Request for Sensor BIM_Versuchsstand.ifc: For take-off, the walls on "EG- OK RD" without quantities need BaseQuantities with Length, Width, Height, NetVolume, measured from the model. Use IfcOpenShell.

First a look at what the model holds.

```python
import ifcopenshell
import ifcopenshell.util.element
import ifcopenshell.util.unit

model = ifcopenshell.open("Sensor BIM_Versuchsstand.ifc")
print(model.schema)
for unit_type in ("LENGTHUNIT", "AREAUNIT", "VOLUMEUNIT"):
    print(unit_type, ifcopenshell.util.unit.calculate_unit_scale(model, unit_type))
storey = next(s for s in model.by_type("IfcBuildingStorey") if s.Name == "EG- OK RD")
walls = [e for e in ifcopenshell.util.element.get_decomposition(storey) if e.is_a("IfcWall")]
for e in sorted(walls, key=lambda e: e.id()):
    print(e.id(), e.is_a(), e.Name, list(ifcopenshell.util.element.get_psets(e, qtos_only=True)), sep=" | ")
```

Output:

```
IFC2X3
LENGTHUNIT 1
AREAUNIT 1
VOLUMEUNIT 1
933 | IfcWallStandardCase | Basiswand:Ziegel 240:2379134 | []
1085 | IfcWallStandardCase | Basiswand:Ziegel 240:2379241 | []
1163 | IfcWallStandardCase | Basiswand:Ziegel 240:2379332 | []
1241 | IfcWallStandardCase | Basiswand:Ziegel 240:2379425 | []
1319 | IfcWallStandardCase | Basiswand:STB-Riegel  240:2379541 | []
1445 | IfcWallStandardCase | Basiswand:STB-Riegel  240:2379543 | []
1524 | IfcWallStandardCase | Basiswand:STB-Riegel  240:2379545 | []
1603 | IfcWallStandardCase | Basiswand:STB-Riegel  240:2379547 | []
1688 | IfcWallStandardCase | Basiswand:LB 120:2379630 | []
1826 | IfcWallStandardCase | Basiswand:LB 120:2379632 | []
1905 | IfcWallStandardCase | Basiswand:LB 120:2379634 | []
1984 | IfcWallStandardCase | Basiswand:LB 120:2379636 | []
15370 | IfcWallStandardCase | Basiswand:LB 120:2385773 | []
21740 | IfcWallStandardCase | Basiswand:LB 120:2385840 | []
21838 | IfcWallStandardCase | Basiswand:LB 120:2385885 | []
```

```python
import ifcopenshell
import ifcopenshell.api.pset
import ifcopenshell.geom
import ifcopenshell.util.element
import ifcopenshell.util.shape
import ifcopenshell.util.unit

model = ifcopenshell.open("Sensor BIM_Versuchsstand.ifc")
unit_scale = ifcopenshell.util.unit.calculate_unit_scale(model)
volume_scale = ifcopenshell.util.unit.calculate_unit_scale(model, "VOLUMEUNIT")
settings = ifcopenshell.geom.settings()

storey = next(s for s in model.by_type("IfcBuildingStorey") if s.Name == "EG- OK RD")
walls = [e for e in ifcopenshell.util.element.get_decomposition(storey) if e.is_a("IfcWall")]

for e in sorted(walls, key=lambda e: e.id()):
    if ifcopenshell.util.element.get_psets(e, qtos_only=True, should_inherit=False):
        continue
    # Geometry comes back in metres, in the element's own axes.
    shape = ifcopenshell.geom.create_shape(settings, e)
    values = {
        "Length": ifcopenshell.util.shape.get_x(shape.geometry) / unit_scale,
        "Width": ifcopenshell.util.shape.get_y(shape.geometry) / unit_scale,
        "Height": ifcopenshell.util.shape.get_z(shape.geometry) / unit_scale,
        "NetVolume": ifcopenshell.util.shape.get_volume(shape.geometry) / volume_scale,
    }
    qto = ifcopenshell.api.pset.add_qto(model, product=e, name="BaseQuantities")
    ifcopenshell.api.pset.edit_qto(model, qto=qto, properties=values)
    print(e.id(), {k: round(v, 3) for k, v in values.items()})

model.write("Sensor BIM_Versuchsstand_rev.ifc")
```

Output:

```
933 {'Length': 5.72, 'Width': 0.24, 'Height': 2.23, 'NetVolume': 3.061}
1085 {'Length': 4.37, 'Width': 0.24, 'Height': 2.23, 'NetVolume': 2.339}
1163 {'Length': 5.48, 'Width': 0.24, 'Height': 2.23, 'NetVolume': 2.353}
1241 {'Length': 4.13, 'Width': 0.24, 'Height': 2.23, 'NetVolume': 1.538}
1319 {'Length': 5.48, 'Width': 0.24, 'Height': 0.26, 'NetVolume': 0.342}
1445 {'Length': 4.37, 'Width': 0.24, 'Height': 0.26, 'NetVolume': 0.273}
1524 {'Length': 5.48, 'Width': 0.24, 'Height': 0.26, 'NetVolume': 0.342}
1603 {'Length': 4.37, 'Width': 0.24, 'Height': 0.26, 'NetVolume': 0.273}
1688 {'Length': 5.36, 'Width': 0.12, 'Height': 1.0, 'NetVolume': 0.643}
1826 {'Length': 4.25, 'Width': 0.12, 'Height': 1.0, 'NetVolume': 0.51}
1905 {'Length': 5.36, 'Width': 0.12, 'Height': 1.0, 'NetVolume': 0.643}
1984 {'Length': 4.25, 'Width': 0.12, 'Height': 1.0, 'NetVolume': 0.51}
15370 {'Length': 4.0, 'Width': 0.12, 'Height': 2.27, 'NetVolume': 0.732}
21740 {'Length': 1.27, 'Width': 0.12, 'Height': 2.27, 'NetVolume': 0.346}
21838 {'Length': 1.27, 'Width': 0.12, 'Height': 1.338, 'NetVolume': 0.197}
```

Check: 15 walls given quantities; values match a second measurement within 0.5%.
